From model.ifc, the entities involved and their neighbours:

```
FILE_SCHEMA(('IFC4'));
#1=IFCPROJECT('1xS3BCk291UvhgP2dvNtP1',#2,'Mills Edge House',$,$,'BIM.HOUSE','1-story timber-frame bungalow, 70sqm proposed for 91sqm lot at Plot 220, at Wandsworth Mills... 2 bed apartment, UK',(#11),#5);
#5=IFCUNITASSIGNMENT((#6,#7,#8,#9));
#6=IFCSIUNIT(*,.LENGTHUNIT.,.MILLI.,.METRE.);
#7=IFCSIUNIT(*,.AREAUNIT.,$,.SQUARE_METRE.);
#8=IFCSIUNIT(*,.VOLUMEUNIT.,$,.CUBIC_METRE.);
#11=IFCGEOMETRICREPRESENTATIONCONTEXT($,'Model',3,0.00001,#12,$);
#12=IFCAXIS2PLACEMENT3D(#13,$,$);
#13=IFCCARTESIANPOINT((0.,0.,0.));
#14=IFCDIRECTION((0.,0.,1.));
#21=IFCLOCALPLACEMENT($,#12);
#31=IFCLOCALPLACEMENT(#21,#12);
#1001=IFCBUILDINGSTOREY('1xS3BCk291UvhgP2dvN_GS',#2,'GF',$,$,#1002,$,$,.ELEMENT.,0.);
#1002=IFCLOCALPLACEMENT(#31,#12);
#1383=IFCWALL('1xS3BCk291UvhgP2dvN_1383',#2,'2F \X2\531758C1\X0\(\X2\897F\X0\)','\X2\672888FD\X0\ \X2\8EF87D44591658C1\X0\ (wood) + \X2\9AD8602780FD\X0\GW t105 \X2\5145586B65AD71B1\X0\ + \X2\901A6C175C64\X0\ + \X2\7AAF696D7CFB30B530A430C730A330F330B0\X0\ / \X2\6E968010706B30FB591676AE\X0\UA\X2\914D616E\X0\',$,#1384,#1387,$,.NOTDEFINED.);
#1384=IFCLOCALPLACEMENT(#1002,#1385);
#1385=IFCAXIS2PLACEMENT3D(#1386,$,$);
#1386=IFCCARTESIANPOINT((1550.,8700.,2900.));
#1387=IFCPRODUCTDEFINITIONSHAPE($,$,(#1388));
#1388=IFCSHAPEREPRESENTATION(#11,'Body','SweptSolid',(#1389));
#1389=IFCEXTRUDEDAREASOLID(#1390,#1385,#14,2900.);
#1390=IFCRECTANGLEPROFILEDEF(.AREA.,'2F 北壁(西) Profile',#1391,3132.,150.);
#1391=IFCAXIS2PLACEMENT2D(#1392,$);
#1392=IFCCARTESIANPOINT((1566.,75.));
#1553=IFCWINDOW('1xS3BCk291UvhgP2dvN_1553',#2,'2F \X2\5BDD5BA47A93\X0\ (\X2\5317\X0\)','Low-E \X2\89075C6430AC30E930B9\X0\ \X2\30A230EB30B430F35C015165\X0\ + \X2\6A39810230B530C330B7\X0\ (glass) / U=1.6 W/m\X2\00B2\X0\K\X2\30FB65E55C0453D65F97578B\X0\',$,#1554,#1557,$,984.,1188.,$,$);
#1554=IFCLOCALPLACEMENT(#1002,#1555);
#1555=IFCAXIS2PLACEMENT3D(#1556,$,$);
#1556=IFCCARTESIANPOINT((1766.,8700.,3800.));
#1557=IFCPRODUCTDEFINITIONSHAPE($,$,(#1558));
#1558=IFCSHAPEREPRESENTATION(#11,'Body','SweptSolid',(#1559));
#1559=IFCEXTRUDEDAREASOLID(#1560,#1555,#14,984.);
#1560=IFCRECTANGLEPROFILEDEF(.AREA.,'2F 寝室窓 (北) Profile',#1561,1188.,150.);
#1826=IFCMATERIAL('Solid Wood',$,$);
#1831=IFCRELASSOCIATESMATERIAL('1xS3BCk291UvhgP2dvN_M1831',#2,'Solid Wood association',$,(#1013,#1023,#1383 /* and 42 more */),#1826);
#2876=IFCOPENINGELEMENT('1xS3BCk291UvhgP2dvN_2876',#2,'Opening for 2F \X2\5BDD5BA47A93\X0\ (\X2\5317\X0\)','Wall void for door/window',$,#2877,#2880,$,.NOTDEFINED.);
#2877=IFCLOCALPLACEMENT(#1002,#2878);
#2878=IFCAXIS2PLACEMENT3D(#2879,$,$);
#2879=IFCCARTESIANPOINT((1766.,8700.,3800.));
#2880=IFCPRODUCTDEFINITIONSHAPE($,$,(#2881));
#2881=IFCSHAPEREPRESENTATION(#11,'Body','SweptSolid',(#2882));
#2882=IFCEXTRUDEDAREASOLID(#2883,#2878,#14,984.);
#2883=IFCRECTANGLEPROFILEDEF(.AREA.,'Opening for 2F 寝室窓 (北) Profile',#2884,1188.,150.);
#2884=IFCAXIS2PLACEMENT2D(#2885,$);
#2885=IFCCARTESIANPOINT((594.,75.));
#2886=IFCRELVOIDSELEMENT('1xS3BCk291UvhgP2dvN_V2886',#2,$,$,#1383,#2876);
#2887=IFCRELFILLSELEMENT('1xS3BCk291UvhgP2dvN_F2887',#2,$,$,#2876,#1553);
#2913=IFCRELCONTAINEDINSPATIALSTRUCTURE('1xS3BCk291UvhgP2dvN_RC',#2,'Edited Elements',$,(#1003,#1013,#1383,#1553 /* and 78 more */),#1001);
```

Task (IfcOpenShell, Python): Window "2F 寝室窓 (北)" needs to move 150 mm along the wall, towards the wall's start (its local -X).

```python
import ifcopenshell
import ifcopenshell.api.geometry
import ifcopenshell.util.placement
import ifcopenshell.util.unit

model = ifcopenshell.open("model.ifc")
unit_scale = ifcopenshell.util.unit.calculate_unit_scale(model)

window = model.by_id(1553)
opening = window.FillsVoids[0].RelatingOpeningElement
wall = opening.VoidsElements[0].RelatingBuildingElement

wall_matrix = ifcopenshell.util.placement.get_local_placement(wall.ObjectPlacement)
shift = wall_matrix[:3, 0] * -0.15 / unit_scale
before = ifcopenshell.util.placement.get_local_placement(window.ObjectPlacement)[:3, 3].copy()

# The window is not placed relative to its opening, so move both.
for product in (opening, window):
    matrix = ifcopenshell.util.placement.get_local_placement(product.ObjectPlacement)
    matrix[:3, 3] += shift
    ifcopenshell.api.geometry.edit_object_placement(model, product=product, matrix=matrix, is_si=False)

after = ifcopenshell.util.placement.get_local_placement(window.ObjectPlacement)[:3, 3]
print("window moved by", (after - before).round(3) + 0.0)

model.write("model_v2.ifc")
```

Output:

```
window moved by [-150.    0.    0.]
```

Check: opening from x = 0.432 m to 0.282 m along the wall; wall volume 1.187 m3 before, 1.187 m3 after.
